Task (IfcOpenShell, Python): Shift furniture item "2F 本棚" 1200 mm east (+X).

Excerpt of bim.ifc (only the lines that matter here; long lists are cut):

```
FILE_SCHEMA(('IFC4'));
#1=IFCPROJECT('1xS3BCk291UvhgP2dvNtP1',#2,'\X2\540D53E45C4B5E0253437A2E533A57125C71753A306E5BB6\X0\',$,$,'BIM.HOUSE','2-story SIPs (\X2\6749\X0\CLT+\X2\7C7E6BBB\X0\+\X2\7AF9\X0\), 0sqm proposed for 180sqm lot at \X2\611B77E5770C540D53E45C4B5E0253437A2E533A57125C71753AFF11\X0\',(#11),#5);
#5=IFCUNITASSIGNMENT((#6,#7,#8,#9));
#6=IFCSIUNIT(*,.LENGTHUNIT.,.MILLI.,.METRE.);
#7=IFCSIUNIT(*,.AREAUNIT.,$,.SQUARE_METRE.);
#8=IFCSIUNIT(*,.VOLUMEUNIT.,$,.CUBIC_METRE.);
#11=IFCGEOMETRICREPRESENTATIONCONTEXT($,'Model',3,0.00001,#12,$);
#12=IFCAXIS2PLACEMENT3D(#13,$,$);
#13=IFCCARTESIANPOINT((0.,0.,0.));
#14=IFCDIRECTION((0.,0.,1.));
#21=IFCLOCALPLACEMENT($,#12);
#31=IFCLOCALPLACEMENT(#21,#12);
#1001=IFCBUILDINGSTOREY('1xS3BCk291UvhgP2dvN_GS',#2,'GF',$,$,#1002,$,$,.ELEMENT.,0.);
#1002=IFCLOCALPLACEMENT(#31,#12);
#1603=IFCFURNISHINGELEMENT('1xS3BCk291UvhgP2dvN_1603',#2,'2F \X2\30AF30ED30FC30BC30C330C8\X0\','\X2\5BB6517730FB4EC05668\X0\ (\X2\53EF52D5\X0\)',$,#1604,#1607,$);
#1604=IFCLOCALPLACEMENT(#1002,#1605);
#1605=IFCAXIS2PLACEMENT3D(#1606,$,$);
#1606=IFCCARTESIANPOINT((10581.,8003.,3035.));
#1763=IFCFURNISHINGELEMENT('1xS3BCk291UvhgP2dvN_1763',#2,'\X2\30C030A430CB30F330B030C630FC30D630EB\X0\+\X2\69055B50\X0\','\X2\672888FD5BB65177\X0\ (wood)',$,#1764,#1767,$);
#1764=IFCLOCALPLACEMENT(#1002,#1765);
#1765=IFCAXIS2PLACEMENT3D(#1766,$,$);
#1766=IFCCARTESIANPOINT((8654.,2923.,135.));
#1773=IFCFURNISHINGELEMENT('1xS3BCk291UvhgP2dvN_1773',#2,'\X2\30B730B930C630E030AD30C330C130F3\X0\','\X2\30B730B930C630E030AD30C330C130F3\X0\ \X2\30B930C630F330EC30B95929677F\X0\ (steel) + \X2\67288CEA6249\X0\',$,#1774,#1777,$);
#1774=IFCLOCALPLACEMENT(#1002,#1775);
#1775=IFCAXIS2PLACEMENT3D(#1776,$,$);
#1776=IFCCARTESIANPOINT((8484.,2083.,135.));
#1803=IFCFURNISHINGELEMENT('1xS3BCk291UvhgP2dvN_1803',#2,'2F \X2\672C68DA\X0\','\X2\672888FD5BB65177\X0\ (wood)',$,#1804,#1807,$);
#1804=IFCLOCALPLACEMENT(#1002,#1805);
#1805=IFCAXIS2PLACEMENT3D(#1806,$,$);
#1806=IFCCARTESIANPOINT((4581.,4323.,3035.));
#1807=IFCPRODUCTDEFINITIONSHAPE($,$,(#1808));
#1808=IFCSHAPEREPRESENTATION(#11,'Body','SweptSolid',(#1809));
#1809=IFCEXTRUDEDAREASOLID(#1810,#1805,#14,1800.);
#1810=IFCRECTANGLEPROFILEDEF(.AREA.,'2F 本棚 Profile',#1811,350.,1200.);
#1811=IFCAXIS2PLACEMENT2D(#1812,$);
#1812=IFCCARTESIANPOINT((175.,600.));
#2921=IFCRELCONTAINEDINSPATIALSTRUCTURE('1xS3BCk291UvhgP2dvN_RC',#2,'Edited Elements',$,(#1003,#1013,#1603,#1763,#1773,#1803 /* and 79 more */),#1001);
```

```python
import ifcopenshell
import ifcopenshell.api.geometry
import ifcopenshell.util.placement

model = ifcopenshell.open("bim.ifc")

item = model.by_guid("1xS3BCk291UvhgP2dvN_1803")
matrix = ifcopenshell.util.placement.get_local_placement(item.ObjectPlacement)
matrix[0, 3] += 1200.0
ifcopenshell.api.geometry.edit_object_placement(model, product=item, matrix=matrix, is_si=False)

print(ifcopenshell.util.placement.get_local_placement(item.ObjectPlacement).round(3) + 0.0)

model.write("bim_v2.ifc")
```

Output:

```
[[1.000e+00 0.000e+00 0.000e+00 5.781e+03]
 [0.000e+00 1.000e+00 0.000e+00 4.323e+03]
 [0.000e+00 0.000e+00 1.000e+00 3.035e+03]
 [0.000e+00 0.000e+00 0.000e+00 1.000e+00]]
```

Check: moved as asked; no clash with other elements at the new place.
